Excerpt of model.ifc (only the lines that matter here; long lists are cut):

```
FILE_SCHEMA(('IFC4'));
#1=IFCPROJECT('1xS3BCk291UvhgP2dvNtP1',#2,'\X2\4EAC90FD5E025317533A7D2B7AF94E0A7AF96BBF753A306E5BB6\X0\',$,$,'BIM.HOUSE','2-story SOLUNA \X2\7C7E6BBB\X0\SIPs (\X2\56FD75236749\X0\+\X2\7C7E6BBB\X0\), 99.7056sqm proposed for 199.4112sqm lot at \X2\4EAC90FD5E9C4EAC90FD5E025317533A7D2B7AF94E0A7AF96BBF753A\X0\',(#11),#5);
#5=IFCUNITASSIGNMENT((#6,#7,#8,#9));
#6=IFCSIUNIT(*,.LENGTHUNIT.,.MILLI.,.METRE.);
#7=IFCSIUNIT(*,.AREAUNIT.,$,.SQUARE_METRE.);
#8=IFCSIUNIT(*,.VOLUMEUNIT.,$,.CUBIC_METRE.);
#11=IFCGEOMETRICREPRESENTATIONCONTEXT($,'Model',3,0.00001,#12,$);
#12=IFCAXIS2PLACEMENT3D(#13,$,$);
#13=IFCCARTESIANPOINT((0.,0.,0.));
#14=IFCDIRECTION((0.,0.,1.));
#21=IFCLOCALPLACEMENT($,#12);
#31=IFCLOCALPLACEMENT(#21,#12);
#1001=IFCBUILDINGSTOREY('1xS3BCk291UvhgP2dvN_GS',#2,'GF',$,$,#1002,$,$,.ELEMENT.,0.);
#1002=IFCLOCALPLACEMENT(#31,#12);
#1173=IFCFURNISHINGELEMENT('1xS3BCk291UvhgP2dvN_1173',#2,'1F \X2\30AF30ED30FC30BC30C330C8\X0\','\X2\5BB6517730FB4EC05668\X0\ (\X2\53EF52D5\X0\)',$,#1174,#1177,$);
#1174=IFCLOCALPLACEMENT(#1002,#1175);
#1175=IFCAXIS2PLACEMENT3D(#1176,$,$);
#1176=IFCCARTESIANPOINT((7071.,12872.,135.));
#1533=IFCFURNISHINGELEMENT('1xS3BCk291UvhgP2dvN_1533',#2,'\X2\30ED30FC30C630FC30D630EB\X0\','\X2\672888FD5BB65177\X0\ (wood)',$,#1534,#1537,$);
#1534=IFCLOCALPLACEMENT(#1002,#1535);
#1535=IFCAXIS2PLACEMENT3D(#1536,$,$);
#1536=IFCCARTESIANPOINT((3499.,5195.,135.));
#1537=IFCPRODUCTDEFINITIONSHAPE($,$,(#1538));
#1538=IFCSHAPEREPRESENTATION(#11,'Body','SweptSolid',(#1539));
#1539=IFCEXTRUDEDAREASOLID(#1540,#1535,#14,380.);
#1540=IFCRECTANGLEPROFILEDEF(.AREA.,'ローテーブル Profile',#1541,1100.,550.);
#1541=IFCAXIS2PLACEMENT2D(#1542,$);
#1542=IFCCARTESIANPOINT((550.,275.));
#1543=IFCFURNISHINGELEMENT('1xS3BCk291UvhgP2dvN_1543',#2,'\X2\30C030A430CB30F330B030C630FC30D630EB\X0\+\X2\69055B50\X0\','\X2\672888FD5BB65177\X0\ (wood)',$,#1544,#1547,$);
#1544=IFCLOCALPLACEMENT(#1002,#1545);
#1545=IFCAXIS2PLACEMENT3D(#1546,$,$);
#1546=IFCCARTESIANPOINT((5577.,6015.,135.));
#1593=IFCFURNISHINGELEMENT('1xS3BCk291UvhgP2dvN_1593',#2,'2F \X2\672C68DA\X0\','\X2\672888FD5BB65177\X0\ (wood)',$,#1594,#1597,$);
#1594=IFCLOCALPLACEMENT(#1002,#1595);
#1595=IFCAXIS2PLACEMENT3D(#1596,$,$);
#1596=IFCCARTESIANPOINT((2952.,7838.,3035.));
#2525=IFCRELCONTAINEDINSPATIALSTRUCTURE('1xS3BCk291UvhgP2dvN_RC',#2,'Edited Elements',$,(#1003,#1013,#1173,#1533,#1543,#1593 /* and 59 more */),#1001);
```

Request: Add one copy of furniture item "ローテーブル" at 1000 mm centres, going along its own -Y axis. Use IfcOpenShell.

```python
import ifcopenshell
import ifcopenshell.api.geometry
import ifcopenshell.api.root
import ifcopenshell.util.element
import ifcopenshell.util.placement
import ifcopenshell.util.unit

model = ifcopenshell.open("model.ifc")
unit_scale = ifcopenshell.util.unit.calculate_unit_scale(model)


def reuse_history(source, copy):
    """copy_class also copies each property set's owner history, people and application; keep the originals."""
    for rel in copy.IsDefinedBy:
        if rel.is_a("IfcRelDefinesByProperties") and (history := rel.RelatingPropertyDefinition.OwnerHistory):
            rel.RelatingPropertyDefinition.OwnerHistory = source.OwnerHistory
            ifcopenshell.util.element.remove_deep2(model, history)


source = model.by_guid("1xS3BCk291UvhgP2dvN_1533")
base = ifcopenshell.util.placement.get_local_placement(source.ObjectPlacement)
step = -base[:3, 1] * 1 / unit_scale

for i in range(1, 2):
    copy = ifcopenshell.api.root.copy_class(model, product=source)
    copy.Representation = ifcopenshell.util.element.copy_deep(
        model, source.Representation, exclude=["IfcGeometricRepresentationContext", "IfcRepresentationMap"]
    )
    reuse_history(source, copy)
    matrix = base.copy()
    matrix[:3, 3] += i * step
    print("added at", matrix[:3, 3].round(3) + 0.0)
    ifcopenshell.api.geometry.edit_object_placement(model, product=copy, matrix=matrix, is_si=False)

model.write("model_v2.ifc")
```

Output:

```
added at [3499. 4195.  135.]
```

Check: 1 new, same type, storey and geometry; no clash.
